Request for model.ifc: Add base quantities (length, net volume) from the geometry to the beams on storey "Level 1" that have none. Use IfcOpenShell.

First a look at what the model holds.

```python
import ifcopenshell
import ifcopenshell.util.element
import ifcopenshell.util.unit

model = ifcopenshell.open("model.ifc")
print(model.schema)
for unit_type in ("LENGTHUNIT", "AREAUNIT", "VOLUMEUNIT"):
    print(unit_type, ifcopenshell.util.unit.calculate_unit_scale(model, unit_type))
storey = next(s for s in model.by_type("IfcBuildingStorey") if s.Name == "Level 1")
beams = [e for e in ifcopenshell.util.element.get_decomposition(storey) if e.is_a("IfcBeam")]
for e in sorted(beams, key=lambda e: e.id()):
    print(e.id(), e.is_a(), e.Name, list(ifcopenshell.util.element.get_psets(e, qtos_only=True)), sep=" | ")
```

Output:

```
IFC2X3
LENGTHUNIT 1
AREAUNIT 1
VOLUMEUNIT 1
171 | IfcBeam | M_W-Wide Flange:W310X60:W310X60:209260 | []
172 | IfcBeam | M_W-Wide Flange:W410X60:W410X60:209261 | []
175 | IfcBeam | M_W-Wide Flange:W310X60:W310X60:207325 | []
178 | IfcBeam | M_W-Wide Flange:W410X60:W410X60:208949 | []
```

```python
import ifcopenshell
import ifcopenshell.api.pset
import ifcopenshell.geom
import ifcopenshell.util.element
import ifcopenshell.util.shape
import ifcopenshell.util.unit

model = ifcopenshell.open("model.ifc")
unit_scale = ifcopenshell.util.unit.calculate_unit_scale(model)
volume_scale = ifcopenshell.util.unit.calculate_unit_scale(model, "VOLUMEUNIT")
settings = ifcopenshell.geom.settings()

storey = next(s for s in model.by_type("IfcBuildingStorey") if s.Name == "Level 1")
beams = [e for e in ifcopenshell.util.element.get_decomposition(storey) if e.is_a("IfcBeam")]

for e in sorted(beams, key=lambda e: e.id()):
    if ifcopenshell.util.element.get_psets(e, qtos_only=True, should_inherit=False):
        continue
    # Geometry comes back in metres, in the element's own axes.
    shape = ifcopenshell.geom.create_shape(settings, e)
    values = {
        "Length": ifcopenshell.util.shape.get_max_xyz(shape.geometry) / unit_scale,
        "NetVolume": ifcopenshell.util.shape.get_volume(shape.geometry) / volume_scale,
    }
    qto = ifcopenshell.api.pset.add_qto(model, product=e, name="BaseQuantities")
    ifcopenshell.api.pset.edit_qto(model, qto=qto, properties=values)
    print(e.id(), {k: round(v, 3) for k, v in values.items()})

model.write("model-out.ifc")
```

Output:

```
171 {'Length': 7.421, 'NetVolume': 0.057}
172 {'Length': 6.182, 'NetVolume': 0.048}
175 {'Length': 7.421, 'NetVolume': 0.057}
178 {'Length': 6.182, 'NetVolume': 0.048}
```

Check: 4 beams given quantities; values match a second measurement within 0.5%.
